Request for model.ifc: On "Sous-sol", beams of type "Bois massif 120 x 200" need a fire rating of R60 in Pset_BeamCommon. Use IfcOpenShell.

First a look at what the model holds.

```python
import ifcopenshell
import ifcopenshell.util.element

model = ifcopenshell.open("model.ifc")
print(model.schema)
storey = next(s for s in model.by_type("IfcBuildingStorey") if s.Name == "Sous-sol")
beams = [e for e in ifcopenshell.util.element.get_decomposition(storey) if e.is_a("IfcBeam")]
seen = {}
for e in beams:
    element_type = ifcopenshell.util.element.get_type(e)
    key = (element_type.Name if element_type != e and element_type else None, ifcopenshell.util.element.get_pset(e, "Pset_BeamCommon", "FireRating"))
    seen[key] = seen.get(key, 0) + 1
for (name, value), count in sorted(seen.items(), key=str):
    print(count, "x", name, "|", value)
```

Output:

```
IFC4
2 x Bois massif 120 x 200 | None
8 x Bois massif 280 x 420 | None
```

```python
import ifcopenshell
import ifcopenshell.api.pset
import ifcopenshell.util.element

model = ifcopenshell.open("model.ifc")

storey = next(s for s in model.by_type("IfcBuildingStorey") if s.Name == "Sous-sol")
beams = [e for e in ifcopenshell.util.element.get_decomposition(storey) if e.is_a("IfcBeam")]

count = 0
for e in beams:
    element_type = ifcopenshell.util.element.get_type(e)
    if element_type in (None, e) or element_type.Name != "Bois massif 120 x 200":
        continue
    # add_pset returns the element's existing set when there is one.
    pset = ifcopenshell.api.pset.add_pset(model, product=e, name="Pset_BeamCommon")
    ifcopenshell.api.pset.edit_pset(model, pset=pset, properties={"FireRating": "R60"})
    count += 1

print(count, "beams updated")

model.write("model_rev.ifc")
```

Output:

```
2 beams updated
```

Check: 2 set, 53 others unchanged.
